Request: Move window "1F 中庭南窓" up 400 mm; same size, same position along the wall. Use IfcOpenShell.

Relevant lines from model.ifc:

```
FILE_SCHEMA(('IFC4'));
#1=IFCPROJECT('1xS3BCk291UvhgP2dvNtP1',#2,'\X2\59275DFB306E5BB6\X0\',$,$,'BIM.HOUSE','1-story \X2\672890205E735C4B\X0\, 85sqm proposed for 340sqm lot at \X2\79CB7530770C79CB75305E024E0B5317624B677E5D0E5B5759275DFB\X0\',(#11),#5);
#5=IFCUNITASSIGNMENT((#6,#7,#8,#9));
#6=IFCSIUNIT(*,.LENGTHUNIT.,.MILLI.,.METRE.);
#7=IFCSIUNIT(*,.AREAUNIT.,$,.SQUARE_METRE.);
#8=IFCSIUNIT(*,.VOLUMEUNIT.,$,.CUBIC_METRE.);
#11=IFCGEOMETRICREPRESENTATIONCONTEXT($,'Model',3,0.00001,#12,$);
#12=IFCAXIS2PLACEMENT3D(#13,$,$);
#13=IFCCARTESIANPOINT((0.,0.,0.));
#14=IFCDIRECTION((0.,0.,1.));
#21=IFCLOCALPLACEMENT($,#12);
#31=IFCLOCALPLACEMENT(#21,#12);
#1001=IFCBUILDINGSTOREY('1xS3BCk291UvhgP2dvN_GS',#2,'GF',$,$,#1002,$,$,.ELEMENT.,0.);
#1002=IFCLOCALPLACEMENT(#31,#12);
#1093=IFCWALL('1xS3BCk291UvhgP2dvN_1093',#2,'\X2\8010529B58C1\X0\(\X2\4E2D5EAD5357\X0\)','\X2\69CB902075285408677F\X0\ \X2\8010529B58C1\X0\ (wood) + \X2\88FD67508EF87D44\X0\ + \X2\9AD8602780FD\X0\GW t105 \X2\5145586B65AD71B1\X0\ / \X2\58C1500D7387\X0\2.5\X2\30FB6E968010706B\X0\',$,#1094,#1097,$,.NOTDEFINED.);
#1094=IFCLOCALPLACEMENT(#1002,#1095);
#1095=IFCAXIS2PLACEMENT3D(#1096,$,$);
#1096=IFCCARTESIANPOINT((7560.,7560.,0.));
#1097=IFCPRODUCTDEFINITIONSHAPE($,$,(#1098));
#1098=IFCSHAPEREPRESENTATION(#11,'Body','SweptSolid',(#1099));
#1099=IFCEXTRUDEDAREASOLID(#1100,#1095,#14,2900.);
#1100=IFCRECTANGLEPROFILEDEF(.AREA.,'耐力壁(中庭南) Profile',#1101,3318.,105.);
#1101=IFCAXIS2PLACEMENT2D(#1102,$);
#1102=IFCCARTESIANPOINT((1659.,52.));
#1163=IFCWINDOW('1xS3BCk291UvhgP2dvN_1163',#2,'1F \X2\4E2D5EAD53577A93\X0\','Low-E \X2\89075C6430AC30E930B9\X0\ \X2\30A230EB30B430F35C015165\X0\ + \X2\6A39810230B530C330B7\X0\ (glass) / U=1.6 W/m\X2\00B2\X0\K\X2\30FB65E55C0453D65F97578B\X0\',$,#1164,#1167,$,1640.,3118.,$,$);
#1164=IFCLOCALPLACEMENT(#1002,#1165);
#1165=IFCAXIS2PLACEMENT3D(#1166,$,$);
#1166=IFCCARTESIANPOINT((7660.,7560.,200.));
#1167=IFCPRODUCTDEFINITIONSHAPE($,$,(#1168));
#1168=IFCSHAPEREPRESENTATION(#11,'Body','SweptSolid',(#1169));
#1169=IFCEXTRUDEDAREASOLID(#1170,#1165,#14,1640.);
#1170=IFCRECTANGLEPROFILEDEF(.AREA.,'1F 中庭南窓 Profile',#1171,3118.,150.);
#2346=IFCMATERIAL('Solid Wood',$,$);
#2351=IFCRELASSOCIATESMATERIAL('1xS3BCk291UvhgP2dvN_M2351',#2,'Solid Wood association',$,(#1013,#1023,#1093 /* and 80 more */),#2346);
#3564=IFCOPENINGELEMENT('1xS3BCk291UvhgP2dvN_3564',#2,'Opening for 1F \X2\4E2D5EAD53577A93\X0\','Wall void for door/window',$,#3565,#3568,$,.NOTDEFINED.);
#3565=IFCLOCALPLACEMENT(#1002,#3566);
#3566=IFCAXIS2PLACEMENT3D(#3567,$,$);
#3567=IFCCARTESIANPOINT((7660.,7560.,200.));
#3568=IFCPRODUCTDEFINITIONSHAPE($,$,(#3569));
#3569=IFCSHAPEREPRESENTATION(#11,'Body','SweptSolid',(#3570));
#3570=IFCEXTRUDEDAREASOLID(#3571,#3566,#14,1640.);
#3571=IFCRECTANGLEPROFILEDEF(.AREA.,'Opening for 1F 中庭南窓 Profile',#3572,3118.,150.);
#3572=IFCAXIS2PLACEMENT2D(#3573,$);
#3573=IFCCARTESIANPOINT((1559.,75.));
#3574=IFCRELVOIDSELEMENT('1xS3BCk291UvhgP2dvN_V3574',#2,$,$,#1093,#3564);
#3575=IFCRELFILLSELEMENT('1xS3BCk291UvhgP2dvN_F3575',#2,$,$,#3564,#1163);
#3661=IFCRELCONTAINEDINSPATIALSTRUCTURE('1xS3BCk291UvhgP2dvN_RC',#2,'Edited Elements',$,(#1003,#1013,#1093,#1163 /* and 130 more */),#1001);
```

```python
import numpy as np
import ifcopenshell
import ifcopenshell.api.geometry
import ifcopenshell.util.placement
import ifcopenshell.util.unit

model = ifcopenshell.open("model.ifc")
unit_scale = ifcopenshell.util.unit.calculate_unit_scale(model)

window = model.by_guid("1xS3BCk291UvhgP2dvN_1163")
opening = window.FillsVoids[0].RelatingOpeningElement
dz = 400.0

shift = np.array([0.0, 0.0, dz])
# The window is not placed relative to its opening, so move both.
for product in (opening, window):
    matrix = ifcopenshell.util.placement.get_local_placement(product.ObjectPlacement)
    matrix[:3, 3] += shift
    ifcopenshell.api.geometry.edit_object_placement(model, product=product, matrix=matrix, is_si=False)

print(f"moved by {dz * unit_scale:+.3f} m")

model.write("model-out.ifc")
```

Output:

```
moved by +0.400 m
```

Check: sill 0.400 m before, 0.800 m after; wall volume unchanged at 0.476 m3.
